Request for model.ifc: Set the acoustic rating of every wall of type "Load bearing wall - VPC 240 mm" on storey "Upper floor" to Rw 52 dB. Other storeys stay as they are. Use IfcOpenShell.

First a look at what the model holds.

```python
import ifcopenshell
import ifcopenshell.util.element

model = ifcopenshell.open("model.ifc")
print(model.schema)
storey = next(s for s in model.by_type("IfcBuildingStorey") if s.Name == "Upper floor")
walls = [e for e in ifcopenshell.util.element.get_decomposition(storey) if e.is_a("IfcWall")]
seen = {}
for e in walls:
    element_type = ifcopenshell.util.element.get_type(e)
    key = (element_type.Name if element_type != e and element_type else None, ifcopenshell.util.element.get_pset(e, "Pset_WallCommon", "AcousticRating"))
    seen[key] = seen.get(key, 0) + 1
for (name, value), count in sorted(seen.items(), key=str):
    print(count, "x", name, "|", value)
```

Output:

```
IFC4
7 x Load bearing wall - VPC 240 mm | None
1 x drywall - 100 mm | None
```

```python
import ifcopenshell
import ifcopenshell.api.pset
import ifcopenshell.util.element

model = ifcopenshell.open("model.ifc")

storey = next(s for s in model.by_type("IfcBuildingStorey") if s.Name == "Upper floor")
walls = [e for e in ifcopenshell.util.element.get_decomposition(storey) if e.is_a("IfcWall")]

count = 0
for e in walls:
    element_type = ifcopenshell.util.element.get_type(e)
    if element_type in (None, e) or element_type.Name != "Load bearing wall - VPC 240 mm":
        continue
    # add_pset returns the element's existing set when there is one.
    pset = ifcopenshell.api.pset.add_pset(model, product=e, name="Pset_WallCommon")
    ifcopenshell.api.pset.edit_pset(model, pset=pset, properties={"AcousticRating": "Rw 52 dB"})
    count += 1

print(count, "walls updated")

model.write("model_edited.ifc")
```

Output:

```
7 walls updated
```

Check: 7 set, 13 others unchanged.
